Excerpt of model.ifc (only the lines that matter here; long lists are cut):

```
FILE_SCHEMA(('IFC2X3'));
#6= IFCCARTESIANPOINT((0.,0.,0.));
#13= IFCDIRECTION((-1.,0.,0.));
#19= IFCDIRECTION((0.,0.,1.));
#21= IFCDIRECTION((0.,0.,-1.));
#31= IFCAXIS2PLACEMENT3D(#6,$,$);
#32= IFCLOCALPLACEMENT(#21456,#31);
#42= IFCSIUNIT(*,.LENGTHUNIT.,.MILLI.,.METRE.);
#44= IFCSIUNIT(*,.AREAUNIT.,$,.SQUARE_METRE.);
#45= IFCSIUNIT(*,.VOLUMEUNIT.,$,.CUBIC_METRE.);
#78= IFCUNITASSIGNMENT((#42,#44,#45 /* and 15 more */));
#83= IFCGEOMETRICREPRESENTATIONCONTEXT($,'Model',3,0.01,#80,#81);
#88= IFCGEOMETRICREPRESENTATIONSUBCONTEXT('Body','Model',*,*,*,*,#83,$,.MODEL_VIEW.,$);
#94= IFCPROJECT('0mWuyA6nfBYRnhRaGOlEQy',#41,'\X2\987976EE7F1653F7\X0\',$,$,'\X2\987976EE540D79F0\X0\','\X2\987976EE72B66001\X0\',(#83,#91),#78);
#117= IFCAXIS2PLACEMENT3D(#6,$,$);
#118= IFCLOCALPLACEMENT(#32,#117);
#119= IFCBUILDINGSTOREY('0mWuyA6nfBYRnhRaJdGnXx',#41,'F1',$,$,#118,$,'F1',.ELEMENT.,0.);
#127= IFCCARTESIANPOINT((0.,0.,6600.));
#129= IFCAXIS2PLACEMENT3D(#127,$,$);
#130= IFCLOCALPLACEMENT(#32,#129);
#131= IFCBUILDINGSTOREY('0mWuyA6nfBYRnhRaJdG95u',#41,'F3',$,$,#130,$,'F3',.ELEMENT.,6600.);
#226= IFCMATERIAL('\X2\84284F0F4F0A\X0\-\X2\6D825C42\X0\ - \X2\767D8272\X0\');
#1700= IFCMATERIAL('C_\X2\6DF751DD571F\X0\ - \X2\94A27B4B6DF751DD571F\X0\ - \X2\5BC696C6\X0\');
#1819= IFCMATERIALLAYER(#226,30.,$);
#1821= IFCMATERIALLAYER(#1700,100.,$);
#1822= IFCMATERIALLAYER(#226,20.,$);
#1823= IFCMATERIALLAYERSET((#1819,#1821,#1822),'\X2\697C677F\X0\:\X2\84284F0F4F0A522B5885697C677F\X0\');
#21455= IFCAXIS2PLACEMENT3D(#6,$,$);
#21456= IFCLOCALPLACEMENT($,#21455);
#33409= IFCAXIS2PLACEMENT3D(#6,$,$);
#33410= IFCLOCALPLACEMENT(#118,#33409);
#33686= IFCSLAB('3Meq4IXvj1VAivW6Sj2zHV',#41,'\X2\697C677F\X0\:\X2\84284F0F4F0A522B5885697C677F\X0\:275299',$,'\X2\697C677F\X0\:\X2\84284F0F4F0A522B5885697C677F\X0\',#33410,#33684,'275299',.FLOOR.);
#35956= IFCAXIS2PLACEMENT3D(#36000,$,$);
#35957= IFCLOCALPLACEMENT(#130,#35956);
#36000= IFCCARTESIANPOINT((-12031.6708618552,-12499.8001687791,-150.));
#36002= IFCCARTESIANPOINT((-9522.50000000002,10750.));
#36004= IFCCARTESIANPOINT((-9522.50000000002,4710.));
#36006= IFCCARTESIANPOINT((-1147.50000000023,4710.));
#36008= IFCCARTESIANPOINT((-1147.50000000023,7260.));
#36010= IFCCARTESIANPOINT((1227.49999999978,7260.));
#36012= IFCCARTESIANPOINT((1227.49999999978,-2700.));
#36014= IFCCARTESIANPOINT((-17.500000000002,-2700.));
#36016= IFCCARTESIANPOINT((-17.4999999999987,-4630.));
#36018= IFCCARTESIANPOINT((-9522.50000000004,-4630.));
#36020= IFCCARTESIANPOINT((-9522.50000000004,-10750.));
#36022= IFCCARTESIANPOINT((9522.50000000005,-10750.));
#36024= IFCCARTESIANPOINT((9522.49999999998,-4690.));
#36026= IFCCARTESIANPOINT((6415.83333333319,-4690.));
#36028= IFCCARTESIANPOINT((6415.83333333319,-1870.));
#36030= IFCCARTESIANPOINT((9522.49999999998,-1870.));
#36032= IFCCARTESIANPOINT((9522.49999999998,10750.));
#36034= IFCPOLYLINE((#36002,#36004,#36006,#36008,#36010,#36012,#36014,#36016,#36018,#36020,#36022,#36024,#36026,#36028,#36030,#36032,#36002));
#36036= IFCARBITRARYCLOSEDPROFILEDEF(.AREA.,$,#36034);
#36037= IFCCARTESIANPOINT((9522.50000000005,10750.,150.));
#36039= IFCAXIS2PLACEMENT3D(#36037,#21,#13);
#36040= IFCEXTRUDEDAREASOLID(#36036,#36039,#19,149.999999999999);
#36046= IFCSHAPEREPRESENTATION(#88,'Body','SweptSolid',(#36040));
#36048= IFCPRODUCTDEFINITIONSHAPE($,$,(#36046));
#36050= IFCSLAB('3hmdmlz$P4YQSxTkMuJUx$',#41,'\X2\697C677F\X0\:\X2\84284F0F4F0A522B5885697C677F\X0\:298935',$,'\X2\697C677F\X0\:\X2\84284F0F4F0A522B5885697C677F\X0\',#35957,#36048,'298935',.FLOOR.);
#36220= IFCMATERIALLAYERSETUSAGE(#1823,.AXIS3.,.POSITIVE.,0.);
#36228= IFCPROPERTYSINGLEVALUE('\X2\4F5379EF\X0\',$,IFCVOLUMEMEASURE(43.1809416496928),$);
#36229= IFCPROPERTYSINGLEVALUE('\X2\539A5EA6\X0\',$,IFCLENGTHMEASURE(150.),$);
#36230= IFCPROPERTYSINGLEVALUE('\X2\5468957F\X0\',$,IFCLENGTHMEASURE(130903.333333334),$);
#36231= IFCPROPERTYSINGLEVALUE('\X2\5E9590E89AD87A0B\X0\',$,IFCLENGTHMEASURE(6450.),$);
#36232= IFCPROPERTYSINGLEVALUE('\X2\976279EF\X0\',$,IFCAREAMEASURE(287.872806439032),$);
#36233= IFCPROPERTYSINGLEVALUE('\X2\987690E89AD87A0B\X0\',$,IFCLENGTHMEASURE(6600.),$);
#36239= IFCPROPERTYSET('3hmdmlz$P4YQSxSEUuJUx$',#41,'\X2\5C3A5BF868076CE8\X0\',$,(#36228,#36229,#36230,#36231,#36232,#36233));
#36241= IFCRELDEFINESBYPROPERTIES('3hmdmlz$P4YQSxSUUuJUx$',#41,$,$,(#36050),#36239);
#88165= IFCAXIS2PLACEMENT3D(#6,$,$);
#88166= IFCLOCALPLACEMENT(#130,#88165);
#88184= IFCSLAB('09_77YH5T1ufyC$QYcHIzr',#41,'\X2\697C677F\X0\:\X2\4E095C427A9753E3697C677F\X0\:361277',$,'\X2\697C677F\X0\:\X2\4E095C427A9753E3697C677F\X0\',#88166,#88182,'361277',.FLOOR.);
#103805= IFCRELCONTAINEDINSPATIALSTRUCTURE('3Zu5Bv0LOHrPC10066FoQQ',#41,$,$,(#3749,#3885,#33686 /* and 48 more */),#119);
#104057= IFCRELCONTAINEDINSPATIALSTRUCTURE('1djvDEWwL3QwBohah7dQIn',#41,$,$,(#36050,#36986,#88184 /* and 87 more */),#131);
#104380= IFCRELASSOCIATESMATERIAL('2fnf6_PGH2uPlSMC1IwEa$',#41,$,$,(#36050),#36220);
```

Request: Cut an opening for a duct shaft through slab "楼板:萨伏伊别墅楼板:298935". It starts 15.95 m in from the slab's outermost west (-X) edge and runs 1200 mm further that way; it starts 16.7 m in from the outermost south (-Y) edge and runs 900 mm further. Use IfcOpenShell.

```python
import numpy as np
import ifcopenshell
import ifcopenshell.api.feature
import ifcopenshell.api.geometry
import ifcopenshell.api.pset
import ifcopenshell.api.root
import ifcopenshell.geom
import ifcopenshell.util.element
import ifcopenshell.util.placement
import ifcopenshell.util.representation
import ifcopenshell.util.shape
import ifcopenshell.util.unit

model = ifcopenshell.open("model.ifc")
unit_scale = ifcopenshell.util.unit.calculate_unit_scale(model)
area_scale = ifcopenshell.util.unit.calculate_unit_scale(model, "AREAUNIT")
volume_scale = ifcopenshell.util.unit.calculate_unit_scale(model, "VOLUMEUNIT")
settings = ifcopenshell.geom.settings()


def volume(element):
    """Net volume in cubic metres, openings subtracted."""
    shape = ifcopenshell.geom.create_shape(settings, element)
    return ifcopenshell.util.shape.get_volume(shape.geometry)


slab = model.by_guid("3hmdmlz$P4YQSxTkMuJUx$")
before = volume(slab)

# Extent in the slab's own axes, in metres. The edges named are its -X and -Y sides.
slab_shape = ifcopenshell.geom.create_shape(settings, slab)
vertices = ifcopenshell.util.shape.get_vertices(slab_shape.geometry)
x_min, y_min, bottom = vertices.min(axis=0)
top = vertices[:, 2].max()

opening = ifcopenshell.api.root.create_entity(model, ifc_class="IfcOpeningElement", name="Duct shaft opening")
context = ifcopenshell.util.representation.get_context(model, "Model", "Body", "MODEL_VIEW")
width, depth = 1.2, 0.9
outline = [(0.0, 0.0), (width, 0.0), (width, depth), (0.0, depth), (0.0, 0.0)]
# Overshoot both faces by 50 mm so the cut is clean.
shape = ifcopenshell.api.geometry.add_slab_representation(
    model, context=context, depth=top - bottom + 0.1, polyline=outline
)
ifcopenshell.api.geometry.assign_representation(model, product=opening, representation=shape)

matrix = ifcopenshell.util.placement.get_local_placement(slab.ObjectPlacement)
matrix[:, 3] = matrix @ np.append(np.array([x_min + 15.95, y_min + 16.7, bottom - 0.05]) / unit_scale, 1.0)
ifcopenshell.api.geometry.edit_object_placement(model, product=opening, matrix=matrix, is_si=False)
ifcopenshell.api.feature.add_feature(model, feature=opening, element=slab)

after = volume(slab)

# Update the slab's stored quantities.
pset = model.by_id(ifcopenshell.util.element.get_pset(slab, "尺寸标注", should_inherit=False)["id"])
ifcopenshell.api.pset.edit_pset(model, pset=pset, properties={
    "体积": model.create_entity("IfcVolumeMeasure", after / volume_scale),
    "面积": model.create_entity("IfcAreaMeasure", after / (top - bottom) / area_scale),
})

print(f"slab volume {before:.3f} -> {after:.3f} m3")

model.write("model-out.ifc")
```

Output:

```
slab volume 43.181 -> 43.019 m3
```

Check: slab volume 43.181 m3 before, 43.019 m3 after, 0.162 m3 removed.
